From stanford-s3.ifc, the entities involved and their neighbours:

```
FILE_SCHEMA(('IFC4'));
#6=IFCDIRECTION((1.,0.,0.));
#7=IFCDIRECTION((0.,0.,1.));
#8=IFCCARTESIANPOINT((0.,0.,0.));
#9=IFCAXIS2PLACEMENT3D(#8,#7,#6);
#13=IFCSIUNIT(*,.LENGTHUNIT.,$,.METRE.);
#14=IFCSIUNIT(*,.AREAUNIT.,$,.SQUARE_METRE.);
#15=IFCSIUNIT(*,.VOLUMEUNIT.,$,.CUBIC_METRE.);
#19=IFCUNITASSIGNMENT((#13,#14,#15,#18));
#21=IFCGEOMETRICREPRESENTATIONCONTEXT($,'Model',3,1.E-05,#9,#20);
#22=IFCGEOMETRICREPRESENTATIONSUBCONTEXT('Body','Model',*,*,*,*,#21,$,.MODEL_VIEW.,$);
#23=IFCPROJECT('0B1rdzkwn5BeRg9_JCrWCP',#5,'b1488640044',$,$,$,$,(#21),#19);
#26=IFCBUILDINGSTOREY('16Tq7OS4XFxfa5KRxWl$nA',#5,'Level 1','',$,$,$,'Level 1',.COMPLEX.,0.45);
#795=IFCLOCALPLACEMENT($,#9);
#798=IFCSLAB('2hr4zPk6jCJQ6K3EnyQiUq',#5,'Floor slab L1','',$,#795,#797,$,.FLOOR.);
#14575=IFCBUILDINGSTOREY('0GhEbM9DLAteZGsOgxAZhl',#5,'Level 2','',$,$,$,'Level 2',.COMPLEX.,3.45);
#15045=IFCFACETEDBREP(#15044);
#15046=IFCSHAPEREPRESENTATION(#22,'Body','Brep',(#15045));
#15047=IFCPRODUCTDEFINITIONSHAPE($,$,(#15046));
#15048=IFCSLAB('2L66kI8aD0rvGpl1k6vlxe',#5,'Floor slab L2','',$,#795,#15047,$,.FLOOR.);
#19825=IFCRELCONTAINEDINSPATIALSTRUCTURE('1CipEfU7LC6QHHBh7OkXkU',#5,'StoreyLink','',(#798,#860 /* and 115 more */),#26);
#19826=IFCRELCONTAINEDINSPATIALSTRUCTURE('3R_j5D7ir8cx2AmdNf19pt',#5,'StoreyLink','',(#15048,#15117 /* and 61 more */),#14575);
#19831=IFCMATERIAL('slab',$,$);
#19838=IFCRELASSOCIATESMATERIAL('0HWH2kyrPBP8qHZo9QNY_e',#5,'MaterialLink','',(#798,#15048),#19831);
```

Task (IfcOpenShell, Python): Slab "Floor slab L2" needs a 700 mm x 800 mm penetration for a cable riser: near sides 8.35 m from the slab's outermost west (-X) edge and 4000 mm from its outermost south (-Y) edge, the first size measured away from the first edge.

```python
import numpy as np
import ifcopenshell
import ifcopenshell.api.feature
import ifcopenshell.api.geometry
import ifcopenshell.api.root
import ifcopenshell.geom
import ifcopenshell.util.placement
import ifcopenshell.util.representation
import ifcopenshell.util.shape
import ifcopenshell.util.unit

model = ifcopenshell.open("stanford-s3.ifc")
unit_scale = ifcopenshell.util.unit.calculate_unit_scale(model)
settings = ifcopenshell.geom.settings()


def volume(element):
    """Net volume in cubic metres, openings subtracted."""
    shape = ifcopenshell.geom.create_shape(settings, element)
    return ifcopenshell.util.shape.get_volume(shape.geometry)


slab = model.by_guid("2L66kI8aD0rvGpl1k6vlxe")
before = volume(slab)

# Extent in the slab's own axes, in metres. The edges named are its -X and -Y sides.
slab_shape = ifcopenshell.geom.create_shape(settings, slab)
vertices = ifcopenshell.util.shape.get_vertices(slab_shape.geometry)
x_min, y_min, bottom = vertices.min(axis=0)
top = vertices[:, 2].max()

opening = ifcopenshell.api.root.create_entity(model, ifc_class="IfcOpeningElement", name="Cable riser opening", predefined_type="OPENING")
context = ifcopenshell.util.representation.get_context(model, "Model", "Body", "MODEL_VIEW")
width, depth = 0.7, 0.8
outline = [(0.0, 0.0), (width, 0.0), (width, depth), (0.0, depth), (0.0, 0.0)]
# Overshoot both faces by 50 mm so the cut is clean.
shape = ifcopenshell.api.geometry.add_slab_representation(
    model, context=context, depth=top - bottom + 0.1, polyline=outline
)
ifcopenshell.api.geometry.assign_representation(model, product=opening, representation=shape)

matrix = ifcopenshell.util.placement.get_local_placement(slab.ObjectPlacement)
matrix[:, 3] = matrix @ np.append(np.array([x_min + 8.35, y_min + 4, bottom - 0.05]) / unit_scale, 1.0)
ifcopenshell.api.geometry.edit_object_placement(model, product=opening, matrix=matrix, is_si=False)
ifcopenshell.api.feature.add_feature(model, feature=opening, element=slab)

after = volume(slab)

print(f"slab volume {before:.3f} -> {after:.3f} m3")

model.write("stanford-s3_edited.ifc")
```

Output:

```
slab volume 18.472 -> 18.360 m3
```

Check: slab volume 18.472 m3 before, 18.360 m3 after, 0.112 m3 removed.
